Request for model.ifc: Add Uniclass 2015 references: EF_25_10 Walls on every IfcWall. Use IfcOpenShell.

First a look at what the model holds.

```python
import ifcopenshell

model = ifcopenshell.open("model.ifc")
print(model.schema)
print("classifications:", [c.Name for c in model.by_type("IfcClassification")])
for ifc_class in ("IfcDoor", "IfcRoof", "IfcStair", "IfcWall", "IfcWindow"):
    print(ifc_class, len(model.by_type(ifc_class)))
```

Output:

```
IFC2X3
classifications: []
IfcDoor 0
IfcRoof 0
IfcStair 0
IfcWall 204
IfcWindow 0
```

```python
import ifcopenshell
import ifcopenshell.api.classification

model = ifcopenshell.open("model.ifc")

# IFC2X3 requires Source and Edition and has no link from the project to the system.
system = model.create_entity("IfcClassification", Source="NBS", Edition="2015", Name="Uniclass 2015")

codes = {
    "IfcWall": ("EF_25_10", "Walls"),
}
for ifc_class, (code, name) in codes.items():
    products = model.by_type(ifc_class)
    ifcopenshell.api.classification.add_reference(
        model, products=products, classification=system, identification=code, name=name
    )
    print(code, len(products))

model.write("model-out.ifc")
```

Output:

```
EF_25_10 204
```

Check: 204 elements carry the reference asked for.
